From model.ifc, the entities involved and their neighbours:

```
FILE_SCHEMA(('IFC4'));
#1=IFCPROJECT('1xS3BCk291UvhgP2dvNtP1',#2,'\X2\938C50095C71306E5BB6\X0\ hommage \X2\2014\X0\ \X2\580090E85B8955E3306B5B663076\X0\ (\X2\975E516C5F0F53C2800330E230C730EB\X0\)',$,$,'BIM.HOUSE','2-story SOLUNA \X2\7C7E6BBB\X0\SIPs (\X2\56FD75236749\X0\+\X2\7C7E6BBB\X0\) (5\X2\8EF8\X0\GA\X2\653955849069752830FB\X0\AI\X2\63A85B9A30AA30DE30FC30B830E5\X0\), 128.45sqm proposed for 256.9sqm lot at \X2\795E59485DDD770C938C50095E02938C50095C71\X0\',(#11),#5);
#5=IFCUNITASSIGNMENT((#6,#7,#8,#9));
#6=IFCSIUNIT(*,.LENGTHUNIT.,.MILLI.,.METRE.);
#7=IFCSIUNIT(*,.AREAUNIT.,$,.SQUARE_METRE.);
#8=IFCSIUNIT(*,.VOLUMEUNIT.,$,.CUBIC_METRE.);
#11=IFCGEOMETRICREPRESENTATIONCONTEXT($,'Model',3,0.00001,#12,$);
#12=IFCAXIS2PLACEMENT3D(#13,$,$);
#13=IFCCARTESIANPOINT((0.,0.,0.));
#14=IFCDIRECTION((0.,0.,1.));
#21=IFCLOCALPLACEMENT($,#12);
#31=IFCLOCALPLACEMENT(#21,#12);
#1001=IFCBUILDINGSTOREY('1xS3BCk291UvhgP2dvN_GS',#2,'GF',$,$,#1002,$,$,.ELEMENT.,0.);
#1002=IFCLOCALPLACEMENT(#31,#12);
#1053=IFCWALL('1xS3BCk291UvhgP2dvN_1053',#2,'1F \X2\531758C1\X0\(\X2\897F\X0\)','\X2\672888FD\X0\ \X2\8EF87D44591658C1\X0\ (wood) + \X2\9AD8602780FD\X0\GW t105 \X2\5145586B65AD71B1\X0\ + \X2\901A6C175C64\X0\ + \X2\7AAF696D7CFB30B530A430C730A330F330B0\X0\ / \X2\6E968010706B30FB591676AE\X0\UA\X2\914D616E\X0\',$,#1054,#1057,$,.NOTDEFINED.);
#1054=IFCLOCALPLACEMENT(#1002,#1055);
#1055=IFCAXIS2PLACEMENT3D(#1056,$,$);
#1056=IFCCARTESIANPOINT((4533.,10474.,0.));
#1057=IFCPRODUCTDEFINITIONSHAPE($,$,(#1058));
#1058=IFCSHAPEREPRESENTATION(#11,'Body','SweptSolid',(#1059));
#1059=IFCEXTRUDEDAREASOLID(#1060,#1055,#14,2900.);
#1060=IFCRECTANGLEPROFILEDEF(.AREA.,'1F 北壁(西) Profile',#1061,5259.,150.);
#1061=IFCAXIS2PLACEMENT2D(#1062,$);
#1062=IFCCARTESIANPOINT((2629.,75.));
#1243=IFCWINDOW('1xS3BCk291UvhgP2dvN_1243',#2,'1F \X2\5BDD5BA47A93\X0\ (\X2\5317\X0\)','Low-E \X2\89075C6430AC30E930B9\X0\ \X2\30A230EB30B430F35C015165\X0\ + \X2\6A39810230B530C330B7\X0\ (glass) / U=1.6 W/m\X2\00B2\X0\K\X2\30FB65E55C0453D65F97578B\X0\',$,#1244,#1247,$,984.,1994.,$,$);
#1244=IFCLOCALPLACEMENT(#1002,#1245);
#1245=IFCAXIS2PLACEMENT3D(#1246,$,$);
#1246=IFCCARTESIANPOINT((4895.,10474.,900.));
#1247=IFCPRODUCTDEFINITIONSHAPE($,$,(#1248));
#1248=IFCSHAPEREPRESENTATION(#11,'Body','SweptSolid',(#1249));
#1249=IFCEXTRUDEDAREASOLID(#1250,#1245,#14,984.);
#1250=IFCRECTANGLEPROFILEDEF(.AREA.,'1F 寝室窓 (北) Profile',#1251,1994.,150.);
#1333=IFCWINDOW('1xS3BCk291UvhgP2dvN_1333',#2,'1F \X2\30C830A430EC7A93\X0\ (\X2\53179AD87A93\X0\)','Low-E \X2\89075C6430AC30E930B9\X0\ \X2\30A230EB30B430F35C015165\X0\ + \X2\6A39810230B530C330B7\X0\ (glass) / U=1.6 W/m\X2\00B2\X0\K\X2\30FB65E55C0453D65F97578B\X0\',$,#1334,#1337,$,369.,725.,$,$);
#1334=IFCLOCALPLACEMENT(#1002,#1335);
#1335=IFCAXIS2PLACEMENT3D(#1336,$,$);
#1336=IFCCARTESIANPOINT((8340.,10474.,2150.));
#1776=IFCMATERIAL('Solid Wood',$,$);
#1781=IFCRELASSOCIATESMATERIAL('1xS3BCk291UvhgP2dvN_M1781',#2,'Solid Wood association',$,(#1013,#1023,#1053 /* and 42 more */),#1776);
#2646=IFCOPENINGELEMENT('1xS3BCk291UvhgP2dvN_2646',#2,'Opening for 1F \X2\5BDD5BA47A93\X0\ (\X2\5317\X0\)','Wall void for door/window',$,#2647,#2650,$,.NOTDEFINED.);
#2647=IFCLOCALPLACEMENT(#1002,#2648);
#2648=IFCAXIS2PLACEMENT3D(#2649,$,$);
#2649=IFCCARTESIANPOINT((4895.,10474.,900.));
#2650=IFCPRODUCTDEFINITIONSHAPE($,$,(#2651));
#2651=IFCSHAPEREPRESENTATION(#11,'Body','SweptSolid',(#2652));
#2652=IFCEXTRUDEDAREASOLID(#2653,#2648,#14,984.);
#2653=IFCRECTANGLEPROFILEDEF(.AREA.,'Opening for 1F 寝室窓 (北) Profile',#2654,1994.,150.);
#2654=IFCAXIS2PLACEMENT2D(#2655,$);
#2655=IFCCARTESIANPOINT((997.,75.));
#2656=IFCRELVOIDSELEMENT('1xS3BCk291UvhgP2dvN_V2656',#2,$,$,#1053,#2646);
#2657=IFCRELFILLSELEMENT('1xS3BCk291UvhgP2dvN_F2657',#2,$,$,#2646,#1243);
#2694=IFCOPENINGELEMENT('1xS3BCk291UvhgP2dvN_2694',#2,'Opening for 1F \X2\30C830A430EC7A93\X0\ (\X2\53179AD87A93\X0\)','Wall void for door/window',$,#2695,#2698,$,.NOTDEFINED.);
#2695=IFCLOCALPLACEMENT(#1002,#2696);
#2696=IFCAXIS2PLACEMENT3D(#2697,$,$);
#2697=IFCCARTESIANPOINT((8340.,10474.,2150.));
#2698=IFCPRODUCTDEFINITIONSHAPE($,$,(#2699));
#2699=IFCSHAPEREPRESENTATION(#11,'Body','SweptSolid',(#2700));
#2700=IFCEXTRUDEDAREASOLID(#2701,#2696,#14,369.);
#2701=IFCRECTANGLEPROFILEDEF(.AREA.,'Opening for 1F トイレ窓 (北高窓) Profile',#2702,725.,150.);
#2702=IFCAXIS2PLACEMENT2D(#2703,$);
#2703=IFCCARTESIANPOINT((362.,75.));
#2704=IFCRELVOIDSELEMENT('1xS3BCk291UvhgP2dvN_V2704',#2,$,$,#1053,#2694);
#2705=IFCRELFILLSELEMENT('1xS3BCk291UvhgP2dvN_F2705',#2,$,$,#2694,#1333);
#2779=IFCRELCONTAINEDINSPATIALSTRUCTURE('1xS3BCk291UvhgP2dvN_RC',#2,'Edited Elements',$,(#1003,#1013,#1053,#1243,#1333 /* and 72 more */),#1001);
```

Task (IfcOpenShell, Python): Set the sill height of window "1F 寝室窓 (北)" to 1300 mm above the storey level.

```python
import numpy as np
import ifcopenshell
import ifcopenshell.api.geometry
import ifcopenshell.geom
import ifcopenshell.util.element
import ifcopenshell.util.placement
import ifcopenshell.util.shape
import ifcopenshell.util.unit

model = ifcopenshell.open("model.ifc")
unit_scale = ifcopenshell.util.unit.calculate_unit_scale(model)

window = model.by_guid("1xS3BCk291UvhgP2dvN_1243")
opening = window.FillsVoids[0].RelatingOpeningElement
storey = ifcopenshell.util.element.get_container(window, ifc_class="IfcBuildingStorey")
level = ifcopenshell.util.placement.get_local_placement(storey.ObjectPlacement)[2, 3]

# The opening's origin need not be at the sill, so measure its lowest point.
shape = ifcopenshell.geom.create_shape(ifcopenshell.geom.settings(), opening)
bottom = ifcopenshell.util.shape.get_shape_bottom_elevation(shape, shape.geometry) / unit_scale
dz = level + 1.3 / unit_scale - bottom

shift = np.array([0.0, 0.0, dz])
# The window is not placed relative to its opening, so move both.
for product in (opening, window):
    matrix = ifcopenshell.util.placement.get_local_placement(product.ObjectPlacement)
    matrix[:3, 3] += shift
    ifcopenshell.api.geometry.edit_object_placement(model, product=product, matrix=matrix, is_si=False)

print(f"moved by {dz * unit_scale:+.3f} m")

model.write("model_rev.ifc")
```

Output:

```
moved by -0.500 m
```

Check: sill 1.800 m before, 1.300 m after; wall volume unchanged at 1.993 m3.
